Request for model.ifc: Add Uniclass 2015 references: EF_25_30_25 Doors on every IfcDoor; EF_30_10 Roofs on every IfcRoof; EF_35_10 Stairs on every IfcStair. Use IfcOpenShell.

First a look at what the model holds.

```python
import ifcopenshell

model = ifcopenshell.open("model.ifc")
print(model.schema)
print("classifications:", [c.Name for c in model.by_type("IfcClassification")])
for ifc_class in ("IfcDoor", "IfcRoof", "IfcStair", "IfcWall", "IfcWindow"):
    print(ifc_class, len(model.by_type(ifc_class)))
```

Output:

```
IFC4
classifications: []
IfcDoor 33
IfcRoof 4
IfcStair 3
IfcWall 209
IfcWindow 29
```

```python
import ifcopenshell
import ifcopenshell.api.classification

model = ifcopenshell.open("model.ifc")

system = ifcopenshell.api.classification.add_classification(model, classification="Uniclass 2015")

codes = {
    "IfcDoor": ("EF_25_30_25", "Doors"),
    "IfcRoof": ("EF_30_10", "Roofs"),
    "IfcStair": ("EF_35_10", "Stairs"),
}
for ifc_class, (code, name) in codes.items():
    products = model.by_type(ifc_class)
    ifcopenshell.api.classification.add_reference(
        model, products=products, classification=system, identification=code, name=name
    )
    print(code, len(products))

model.write("model_v2.ifc")
```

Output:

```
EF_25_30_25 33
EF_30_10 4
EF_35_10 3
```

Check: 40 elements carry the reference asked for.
